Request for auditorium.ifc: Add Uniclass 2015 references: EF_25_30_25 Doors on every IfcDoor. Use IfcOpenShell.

First a look at what the model holds.

```python
import ifcopenshell

model = ifcopenshell.open("auditorium.ifc")
print(model.schema)
print("classifications:", [c.Name for c in model.by_type("IfcClassification")])
for ifc_class in ("IfcDoor", "IfcRoof", "IfcStair", "IfcWall", "IfcWindow"):
    print(ifc_class, len(model.by_type(ifc_class)))
```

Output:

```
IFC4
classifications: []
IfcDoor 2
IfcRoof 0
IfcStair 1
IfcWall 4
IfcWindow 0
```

```python
import ifcopenshell
import ifcopenshell.api.classification

model = ifcopenshell.open("auditorium.ifc")

system = ifcopenshell.api.classification.add_classification(model, classification="Uniclass 2015")

codes = {
    "IfcDoor": ("EF_25_30_25", "Doors"),
}
for ifc_class, (code, name) in codes.items():
    products = model.by_type(ifc_class)
    ifcopenshell.api.classification.add_reference(
        model, products=products, classification=system, identification=code, name=name
    )
    print(code, len(products))

model.write("auditorium_edited.ifc")
```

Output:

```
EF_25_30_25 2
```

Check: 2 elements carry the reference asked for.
